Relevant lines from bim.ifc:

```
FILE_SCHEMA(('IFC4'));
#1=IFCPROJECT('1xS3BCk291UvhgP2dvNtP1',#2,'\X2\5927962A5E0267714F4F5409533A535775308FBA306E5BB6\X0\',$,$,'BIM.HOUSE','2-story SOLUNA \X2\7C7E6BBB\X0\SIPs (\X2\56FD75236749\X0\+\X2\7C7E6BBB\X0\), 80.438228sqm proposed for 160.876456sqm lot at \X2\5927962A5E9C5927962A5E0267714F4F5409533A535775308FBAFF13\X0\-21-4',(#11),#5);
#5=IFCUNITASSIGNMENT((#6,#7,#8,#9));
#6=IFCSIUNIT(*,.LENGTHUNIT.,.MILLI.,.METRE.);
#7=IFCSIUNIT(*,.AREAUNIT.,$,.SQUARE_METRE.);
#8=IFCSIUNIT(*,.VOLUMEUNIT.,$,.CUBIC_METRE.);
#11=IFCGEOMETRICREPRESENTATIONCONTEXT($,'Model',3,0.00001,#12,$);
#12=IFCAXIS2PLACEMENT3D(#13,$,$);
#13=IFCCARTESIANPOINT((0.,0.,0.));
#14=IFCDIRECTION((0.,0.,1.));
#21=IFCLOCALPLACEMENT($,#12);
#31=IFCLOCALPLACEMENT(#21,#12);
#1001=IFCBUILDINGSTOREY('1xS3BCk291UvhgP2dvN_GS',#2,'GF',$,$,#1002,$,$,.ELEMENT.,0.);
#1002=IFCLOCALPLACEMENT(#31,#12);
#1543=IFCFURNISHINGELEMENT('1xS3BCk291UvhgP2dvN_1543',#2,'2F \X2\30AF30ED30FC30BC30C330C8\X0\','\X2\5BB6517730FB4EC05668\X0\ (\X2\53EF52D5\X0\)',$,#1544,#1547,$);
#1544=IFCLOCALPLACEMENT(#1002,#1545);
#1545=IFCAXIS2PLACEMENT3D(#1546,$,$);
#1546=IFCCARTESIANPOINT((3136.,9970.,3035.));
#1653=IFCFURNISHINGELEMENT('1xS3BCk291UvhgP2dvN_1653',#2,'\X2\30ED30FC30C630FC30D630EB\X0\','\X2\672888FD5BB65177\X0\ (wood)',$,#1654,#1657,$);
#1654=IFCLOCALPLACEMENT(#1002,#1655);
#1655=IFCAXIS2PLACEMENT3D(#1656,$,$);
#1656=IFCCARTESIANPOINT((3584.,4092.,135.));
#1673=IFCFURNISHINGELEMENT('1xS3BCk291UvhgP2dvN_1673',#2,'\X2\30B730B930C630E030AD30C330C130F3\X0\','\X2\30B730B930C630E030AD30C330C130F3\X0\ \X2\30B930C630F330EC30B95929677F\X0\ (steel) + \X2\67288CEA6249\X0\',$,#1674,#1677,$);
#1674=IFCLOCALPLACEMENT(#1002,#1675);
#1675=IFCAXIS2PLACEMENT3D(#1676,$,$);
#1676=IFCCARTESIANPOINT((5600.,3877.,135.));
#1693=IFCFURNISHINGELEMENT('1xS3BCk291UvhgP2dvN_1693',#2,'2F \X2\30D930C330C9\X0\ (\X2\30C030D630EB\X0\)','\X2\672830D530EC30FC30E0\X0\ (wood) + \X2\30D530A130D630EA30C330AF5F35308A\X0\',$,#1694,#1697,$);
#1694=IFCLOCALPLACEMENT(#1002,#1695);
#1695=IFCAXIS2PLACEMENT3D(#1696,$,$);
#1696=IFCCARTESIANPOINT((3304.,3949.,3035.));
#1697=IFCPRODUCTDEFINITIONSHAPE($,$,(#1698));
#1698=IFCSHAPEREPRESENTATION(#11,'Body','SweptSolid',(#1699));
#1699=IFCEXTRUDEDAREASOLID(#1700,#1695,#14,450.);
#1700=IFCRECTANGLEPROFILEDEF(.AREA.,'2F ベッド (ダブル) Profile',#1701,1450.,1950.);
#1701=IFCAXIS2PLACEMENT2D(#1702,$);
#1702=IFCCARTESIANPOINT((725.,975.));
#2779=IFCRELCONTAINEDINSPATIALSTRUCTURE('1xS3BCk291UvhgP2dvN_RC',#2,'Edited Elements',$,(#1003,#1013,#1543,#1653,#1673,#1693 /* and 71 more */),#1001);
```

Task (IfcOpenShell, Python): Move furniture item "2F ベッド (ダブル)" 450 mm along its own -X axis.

```python
import ifcopenshell
import ifcopenshell.api.geometry
import ifcopenshell.util.placement
import ifcopenshell.util.unit

model = ifcopenshell.open("bim.ifc")
unit_scale = ifcopenshell.util.unit.calculate_unit_scale(model)

item = model.by_guid("1xS3BCk291UvhgP2dvN_1693")
matrix = ifcopenshell.util.placement.get_local_placement(item.ObjectPlacement)
matrix[:3, 3] -= matrix[:3, 0] * 0.45 / unit_scale
ifcopenshell.api.geometry.edit_object_placement(model, product=item, matrix=matrix, is_si=False)

print(ifcopenshell.util.placement.get_local_placement(item.ObjectPlacement).round(3) + 0.0)

model.write("bim_edited.ifc")
```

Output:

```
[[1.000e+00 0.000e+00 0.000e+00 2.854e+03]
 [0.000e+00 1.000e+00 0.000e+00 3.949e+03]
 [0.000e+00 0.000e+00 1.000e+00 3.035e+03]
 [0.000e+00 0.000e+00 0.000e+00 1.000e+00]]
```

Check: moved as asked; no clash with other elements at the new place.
